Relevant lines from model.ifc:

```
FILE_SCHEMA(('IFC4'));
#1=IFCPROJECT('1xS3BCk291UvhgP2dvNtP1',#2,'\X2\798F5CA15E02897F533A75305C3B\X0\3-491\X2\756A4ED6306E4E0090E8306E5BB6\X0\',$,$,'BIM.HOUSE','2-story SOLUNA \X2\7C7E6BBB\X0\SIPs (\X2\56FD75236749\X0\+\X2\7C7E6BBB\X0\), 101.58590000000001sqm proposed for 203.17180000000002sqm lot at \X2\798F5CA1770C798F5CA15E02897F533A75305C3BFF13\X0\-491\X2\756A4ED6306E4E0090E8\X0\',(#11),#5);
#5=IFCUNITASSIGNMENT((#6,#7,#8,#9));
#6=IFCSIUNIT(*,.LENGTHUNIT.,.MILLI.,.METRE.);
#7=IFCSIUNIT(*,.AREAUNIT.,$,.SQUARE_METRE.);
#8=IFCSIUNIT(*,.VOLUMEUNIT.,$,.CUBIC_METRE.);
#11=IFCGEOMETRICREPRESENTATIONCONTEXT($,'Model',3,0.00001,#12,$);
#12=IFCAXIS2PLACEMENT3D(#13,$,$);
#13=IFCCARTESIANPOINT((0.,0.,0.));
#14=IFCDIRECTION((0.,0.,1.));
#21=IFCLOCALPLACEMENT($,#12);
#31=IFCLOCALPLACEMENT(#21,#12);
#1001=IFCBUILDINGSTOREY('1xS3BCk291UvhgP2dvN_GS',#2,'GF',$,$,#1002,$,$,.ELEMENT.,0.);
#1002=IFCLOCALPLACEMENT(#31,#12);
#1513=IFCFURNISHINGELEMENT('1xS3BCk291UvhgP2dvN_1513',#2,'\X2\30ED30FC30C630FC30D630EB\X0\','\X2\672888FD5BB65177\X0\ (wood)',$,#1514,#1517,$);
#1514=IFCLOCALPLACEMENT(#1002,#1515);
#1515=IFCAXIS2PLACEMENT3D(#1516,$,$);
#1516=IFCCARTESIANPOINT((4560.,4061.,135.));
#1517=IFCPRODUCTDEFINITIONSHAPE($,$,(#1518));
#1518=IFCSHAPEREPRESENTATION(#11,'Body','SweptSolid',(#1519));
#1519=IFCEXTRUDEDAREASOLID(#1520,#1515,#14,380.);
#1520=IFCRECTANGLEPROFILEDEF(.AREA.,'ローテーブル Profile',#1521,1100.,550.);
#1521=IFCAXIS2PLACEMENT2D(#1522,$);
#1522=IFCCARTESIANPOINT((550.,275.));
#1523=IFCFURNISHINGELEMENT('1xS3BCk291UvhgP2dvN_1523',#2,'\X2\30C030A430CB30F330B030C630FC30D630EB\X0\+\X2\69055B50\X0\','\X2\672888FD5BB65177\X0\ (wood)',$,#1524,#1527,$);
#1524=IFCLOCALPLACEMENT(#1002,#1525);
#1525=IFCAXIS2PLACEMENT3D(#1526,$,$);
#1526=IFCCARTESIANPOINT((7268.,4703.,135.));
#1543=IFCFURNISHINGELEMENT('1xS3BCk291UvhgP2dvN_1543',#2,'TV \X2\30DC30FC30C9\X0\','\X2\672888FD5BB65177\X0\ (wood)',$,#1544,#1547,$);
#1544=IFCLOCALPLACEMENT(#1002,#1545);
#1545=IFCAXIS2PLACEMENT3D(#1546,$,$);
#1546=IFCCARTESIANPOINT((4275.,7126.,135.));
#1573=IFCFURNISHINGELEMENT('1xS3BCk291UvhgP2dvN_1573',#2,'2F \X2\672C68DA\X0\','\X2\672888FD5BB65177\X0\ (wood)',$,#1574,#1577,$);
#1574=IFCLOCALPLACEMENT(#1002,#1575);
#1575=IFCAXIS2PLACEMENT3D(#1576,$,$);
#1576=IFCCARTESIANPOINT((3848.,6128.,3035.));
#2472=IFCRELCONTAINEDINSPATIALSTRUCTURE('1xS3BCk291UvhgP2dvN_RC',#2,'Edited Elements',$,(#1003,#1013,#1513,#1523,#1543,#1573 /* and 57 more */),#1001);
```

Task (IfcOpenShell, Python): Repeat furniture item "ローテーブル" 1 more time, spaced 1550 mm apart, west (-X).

```python
import numpy as np
import ifcopenshell
import ifcopenshell.api.geometry
import ifcopenshell.api.root
import ifcopenshell.util.element
import ifcopenshell.util.placement
import ifcopenshell.util.unit

model = ifcopenshell.open("model.ifc")
unit_scale = ifcopenshell.util.unit.calculate_unit_scale(model)


def reuse_history(source, copy):
    """copy_class also copies each property set's owner history, people and application; keep the originals."""
    for rel in copy.IsDefinedBy:
        if rel.is_a("IfcRelDefinesByProperties") and (history := rel.RelatingPropertyDefinition.OwnerHistory):
            rel.RelatingPropertyDefinition.OwnerHistory = source.OwnerHistory
            ifcopenshell.util.element.remove_deep2(model, history)


source = model.by_guid("1xS3BCk291UvhgP2dvN_1513")
base = ifcopenshell.util.placement.get_local_placement(source.ObjectPlacement)
step = np.array([-1.0, 0.0, 0.0]) * 1.55 / unit_scale

for i in range(1, 2):
    copy = ifcopenshell.api.root.copy_class(model, product=source)
    copy.Representation = ifcopenshell.util.element.copy_deep(
        model, source.Representation, exclude=["IfcGeometricRepresentationContext", "IfcRepresentationMap"]
    )
    reuse_history(source, copy)
    matrix = base.copy()
    matrix[:3, 3] += i * step
    print("added at", matrix[:3, 3].round(3) + 0.0)
    ifcopenshell.api.geometry.edit_object_placement(model, product=copy, matrix=matrix, is_si=False)

model.write("model_v2.ifc")
```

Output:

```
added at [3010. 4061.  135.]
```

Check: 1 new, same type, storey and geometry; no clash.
